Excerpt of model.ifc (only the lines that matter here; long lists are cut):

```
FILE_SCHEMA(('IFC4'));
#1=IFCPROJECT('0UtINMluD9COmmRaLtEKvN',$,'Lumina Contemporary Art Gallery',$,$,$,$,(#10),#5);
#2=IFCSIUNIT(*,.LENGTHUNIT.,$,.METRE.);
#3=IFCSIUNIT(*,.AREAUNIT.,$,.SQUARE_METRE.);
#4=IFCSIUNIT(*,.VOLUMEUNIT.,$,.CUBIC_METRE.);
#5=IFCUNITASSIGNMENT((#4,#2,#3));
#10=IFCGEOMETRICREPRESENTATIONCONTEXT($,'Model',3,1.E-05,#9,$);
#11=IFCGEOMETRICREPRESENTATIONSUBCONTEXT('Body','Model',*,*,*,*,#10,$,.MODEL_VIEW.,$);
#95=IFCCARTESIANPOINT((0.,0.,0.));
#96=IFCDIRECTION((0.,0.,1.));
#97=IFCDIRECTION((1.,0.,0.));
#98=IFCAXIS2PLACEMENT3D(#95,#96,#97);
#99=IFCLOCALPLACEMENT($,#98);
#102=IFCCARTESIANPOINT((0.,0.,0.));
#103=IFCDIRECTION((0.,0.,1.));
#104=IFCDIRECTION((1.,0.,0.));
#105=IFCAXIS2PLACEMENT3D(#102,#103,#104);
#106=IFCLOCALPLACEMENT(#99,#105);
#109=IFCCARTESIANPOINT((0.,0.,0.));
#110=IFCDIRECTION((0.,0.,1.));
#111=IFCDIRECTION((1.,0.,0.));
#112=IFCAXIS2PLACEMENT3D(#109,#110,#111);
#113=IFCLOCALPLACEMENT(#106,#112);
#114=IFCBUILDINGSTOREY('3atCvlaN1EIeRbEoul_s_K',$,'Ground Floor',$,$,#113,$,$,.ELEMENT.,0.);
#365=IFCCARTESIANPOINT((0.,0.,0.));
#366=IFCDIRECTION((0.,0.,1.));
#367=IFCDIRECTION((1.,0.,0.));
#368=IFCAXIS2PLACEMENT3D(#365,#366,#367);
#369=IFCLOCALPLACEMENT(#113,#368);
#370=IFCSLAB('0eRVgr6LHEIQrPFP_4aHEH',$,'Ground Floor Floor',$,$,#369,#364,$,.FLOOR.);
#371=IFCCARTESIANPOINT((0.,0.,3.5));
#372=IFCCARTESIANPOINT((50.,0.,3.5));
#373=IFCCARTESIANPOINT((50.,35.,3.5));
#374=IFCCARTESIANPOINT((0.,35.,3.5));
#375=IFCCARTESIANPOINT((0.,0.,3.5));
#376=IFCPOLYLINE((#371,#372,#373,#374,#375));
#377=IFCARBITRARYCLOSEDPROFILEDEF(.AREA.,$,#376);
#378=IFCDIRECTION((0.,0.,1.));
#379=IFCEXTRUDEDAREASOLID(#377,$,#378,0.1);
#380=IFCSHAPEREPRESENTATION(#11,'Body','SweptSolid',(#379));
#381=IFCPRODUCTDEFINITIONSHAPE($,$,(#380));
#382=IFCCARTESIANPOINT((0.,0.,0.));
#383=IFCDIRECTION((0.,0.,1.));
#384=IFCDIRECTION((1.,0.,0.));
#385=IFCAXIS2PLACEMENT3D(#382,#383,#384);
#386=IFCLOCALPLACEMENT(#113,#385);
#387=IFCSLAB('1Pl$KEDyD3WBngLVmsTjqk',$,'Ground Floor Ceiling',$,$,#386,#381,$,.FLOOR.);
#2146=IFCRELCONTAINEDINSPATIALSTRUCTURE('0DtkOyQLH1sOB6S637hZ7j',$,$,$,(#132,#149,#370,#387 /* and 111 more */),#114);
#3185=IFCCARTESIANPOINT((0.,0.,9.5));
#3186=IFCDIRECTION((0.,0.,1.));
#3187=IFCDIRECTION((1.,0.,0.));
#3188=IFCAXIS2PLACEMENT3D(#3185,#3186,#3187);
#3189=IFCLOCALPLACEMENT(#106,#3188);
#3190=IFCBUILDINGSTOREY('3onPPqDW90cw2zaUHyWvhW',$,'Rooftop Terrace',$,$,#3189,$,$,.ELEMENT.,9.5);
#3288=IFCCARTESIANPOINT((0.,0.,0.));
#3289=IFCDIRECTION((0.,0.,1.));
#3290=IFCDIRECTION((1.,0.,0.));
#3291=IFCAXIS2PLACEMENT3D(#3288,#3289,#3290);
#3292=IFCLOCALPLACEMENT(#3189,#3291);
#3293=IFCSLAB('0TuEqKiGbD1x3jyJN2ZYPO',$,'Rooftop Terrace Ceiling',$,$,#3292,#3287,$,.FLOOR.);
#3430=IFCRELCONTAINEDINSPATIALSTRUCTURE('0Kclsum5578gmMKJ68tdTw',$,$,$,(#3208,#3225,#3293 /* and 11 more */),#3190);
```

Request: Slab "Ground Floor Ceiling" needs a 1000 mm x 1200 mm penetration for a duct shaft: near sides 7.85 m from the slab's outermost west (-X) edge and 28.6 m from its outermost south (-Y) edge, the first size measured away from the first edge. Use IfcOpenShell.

```python
import numpy as np
import ifcopenshell
import ifcopenshell.api.feature
import ifcopenshell.api.geometry
import ifcopenshell.api.root
import ifcopenshell.geom
import ifcopenshell.util.placement
import ifcopenshell.util.representation
import ifcopenshell.util.shape
import ifcopenshell.util.unit

model = ifcopenshell.open("model.ifc")
unit_scale = ifcopenshell.util.unit.calculate_unit_scale(model)
settings = ifcopenshell.geom.settings()


def volume(element):
    """Net volume in cubic metres, openings subtracted."""
    shape = ifcopenshell.geom.create_shape(settings, element)
    return ifcopenshell.util.shape.get_volume(shape.geometry)


slab = model.by_guid("1Pl$KEDyD3WBngLVmsTjqk")
before = volume(slab)

# Extent in the slab's own axes, in metres. The edges named are its -X and -Y sides.
slab_shape = ifcopenshell.geom.create_shape(settings, slab)
vertices = ifcopenshell.util.shape.get_vertices(slab_shape.geometry)
x_min, y_min, bottom = vertices.min(axis=0)
top = vertices[:, 2].max()

opening = ifcopenshell.api.root.create_entity(model, ifc_class="IfcOpeningElement", name="Duct shaft opening", predefined_type="OPENING")
context = ifcopenshell.util.representation.get_context(model, "Model", "Body", "MODEL_VIEW")
width, depth = 1, 1.2
outline = [(0.0, 0.0), (width, 0.0), (width, depth), (0.0, depth), (0.0, 0.0)]
# Overshoot both faces by 50 mm so the cut is clean.
shape = ifcopenshell.api.geometry.add_slab_representation(
    model, context=context, depth=top - bottom + 0.1, polyline=outline
)
ifcopenshell.api.geometry.assign_representation(model, product=opening, representation=shape)

matrix = ifcopenshell.util.placement.get_local_placement(slab.ObjectPlacement)
matrix[:, 3] = matrix @ np.append(np.array([x_min + 7.85, y_min + 28.6, bottom - 0.05]) / unit_scale, 1.0)
ifcopenshell.api.geometry.edit_object_placement(model, product=opening, matrix=matrix, is_si=False)
ifcopenshell.api.feature.add_feature(model, feature=opening, element=slab)

after = volume(slab)

print(f"slab volume {before:.3f} -> {after:.3f} m3")

model.write("model_v2.ifc")
```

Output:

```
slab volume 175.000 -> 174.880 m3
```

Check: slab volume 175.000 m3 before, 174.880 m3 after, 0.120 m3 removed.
